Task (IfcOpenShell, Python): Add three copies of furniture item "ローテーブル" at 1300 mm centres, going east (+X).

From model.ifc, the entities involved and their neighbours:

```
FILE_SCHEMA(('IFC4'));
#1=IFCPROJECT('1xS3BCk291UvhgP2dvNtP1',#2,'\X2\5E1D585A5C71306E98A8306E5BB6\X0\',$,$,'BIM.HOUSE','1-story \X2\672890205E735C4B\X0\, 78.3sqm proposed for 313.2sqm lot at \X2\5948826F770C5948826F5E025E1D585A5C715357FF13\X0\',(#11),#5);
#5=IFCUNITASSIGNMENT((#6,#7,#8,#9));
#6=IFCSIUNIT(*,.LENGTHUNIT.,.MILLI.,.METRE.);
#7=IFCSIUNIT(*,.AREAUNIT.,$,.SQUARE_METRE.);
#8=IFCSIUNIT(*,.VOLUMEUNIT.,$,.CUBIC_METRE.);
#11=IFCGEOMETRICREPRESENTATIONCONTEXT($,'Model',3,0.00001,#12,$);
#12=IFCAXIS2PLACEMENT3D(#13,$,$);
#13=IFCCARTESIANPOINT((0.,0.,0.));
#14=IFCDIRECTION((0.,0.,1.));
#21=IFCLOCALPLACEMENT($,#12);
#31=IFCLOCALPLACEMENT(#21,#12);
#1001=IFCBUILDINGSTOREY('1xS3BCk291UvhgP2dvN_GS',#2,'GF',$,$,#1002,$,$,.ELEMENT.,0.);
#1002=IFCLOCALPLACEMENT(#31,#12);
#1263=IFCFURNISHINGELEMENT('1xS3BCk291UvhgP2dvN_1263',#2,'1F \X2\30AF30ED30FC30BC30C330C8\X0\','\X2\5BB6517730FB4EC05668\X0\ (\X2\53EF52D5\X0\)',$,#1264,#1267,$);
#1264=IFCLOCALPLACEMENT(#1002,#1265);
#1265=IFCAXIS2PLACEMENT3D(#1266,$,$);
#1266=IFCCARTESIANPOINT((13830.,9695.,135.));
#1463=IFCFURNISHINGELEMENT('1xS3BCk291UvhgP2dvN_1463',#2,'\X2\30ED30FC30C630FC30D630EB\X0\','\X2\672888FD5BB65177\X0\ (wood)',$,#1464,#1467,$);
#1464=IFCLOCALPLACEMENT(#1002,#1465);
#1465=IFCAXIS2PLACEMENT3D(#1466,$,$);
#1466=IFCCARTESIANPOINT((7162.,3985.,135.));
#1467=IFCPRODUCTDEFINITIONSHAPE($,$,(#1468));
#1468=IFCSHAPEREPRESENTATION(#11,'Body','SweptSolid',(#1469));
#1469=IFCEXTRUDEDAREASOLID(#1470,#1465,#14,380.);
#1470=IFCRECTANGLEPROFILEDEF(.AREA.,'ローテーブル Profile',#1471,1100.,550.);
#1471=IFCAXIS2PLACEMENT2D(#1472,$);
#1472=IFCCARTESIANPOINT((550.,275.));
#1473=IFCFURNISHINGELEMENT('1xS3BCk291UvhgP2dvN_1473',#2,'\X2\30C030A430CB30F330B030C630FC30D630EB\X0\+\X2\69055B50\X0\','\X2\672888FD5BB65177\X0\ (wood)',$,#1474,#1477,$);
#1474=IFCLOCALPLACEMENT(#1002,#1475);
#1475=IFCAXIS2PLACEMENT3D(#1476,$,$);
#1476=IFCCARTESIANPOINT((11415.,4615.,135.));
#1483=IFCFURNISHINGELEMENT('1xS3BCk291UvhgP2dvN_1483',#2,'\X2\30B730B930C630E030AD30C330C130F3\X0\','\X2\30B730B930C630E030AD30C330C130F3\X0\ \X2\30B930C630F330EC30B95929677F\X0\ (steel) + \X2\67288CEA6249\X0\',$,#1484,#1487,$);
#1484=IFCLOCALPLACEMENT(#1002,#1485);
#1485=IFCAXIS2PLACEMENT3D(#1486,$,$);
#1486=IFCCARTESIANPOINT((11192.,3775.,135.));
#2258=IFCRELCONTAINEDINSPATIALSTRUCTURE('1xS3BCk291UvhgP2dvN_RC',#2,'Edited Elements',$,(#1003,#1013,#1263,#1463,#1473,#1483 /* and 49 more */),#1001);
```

```python
import numpy as np
import ifcopenshell
import ifcopenshell.api.geometry
import ifcopenshell.api.root
import ifcopenshell.util.element
import ifcopenshell.util.placement

model = ifcopenshell.open("model.ifc")


def reuse_history(source, copy):
    """copy_class also copies each property set's owner history, people and application; keep the originals."""
    for rel in copy.IsDefinedBy:
        if rel.is_a("IfcRelDefinesByProperties") and (history := rel.RelatingPropertyDefinition.OwnerHistory):
            rel.RelatingPropertyDefinition.OwnerHistory = source.OwnerHistory
            ifcopenshell.util.element.remove_deep2(model, history)


source = model.by_guid("1xS3BCk291UvhgP2dvN_1463")
base = ifcopenshell.util.placement.get_local_placement(source.ObjectPlacement)
step = np.array([1.0, 0.0, 0.0]) * 1300.0

for i in range(1, 4):
    copy = ifcopenshell.api.root.copy_class(model, product=source)
    copy.Representation = ifcopenshell.util.element.copy_deep(
        model, source.Representation, exclude=["IfcGeometricRepresentationContext", "IfcRepresentationMap"]
    )
    reuse_history(source, copy)
    matrix = base.copy()
    matrix[:3, 3] += i * step
    print("added at", matrix[:3, 3].round(3) + 0.0)
    ifcopenshell.api.geometry.edit_object_placement(model, product=copy, matrix=matrix, is_si=False)

model.write("model_updated.ifc")
```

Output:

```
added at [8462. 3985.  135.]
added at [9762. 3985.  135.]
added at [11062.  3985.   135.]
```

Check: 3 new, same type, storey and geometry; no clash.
